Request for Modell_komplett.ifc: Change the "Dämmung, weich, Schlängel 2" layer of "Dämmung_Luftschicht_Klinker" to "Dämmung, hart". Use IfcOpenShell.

First a look at what the model holds.

```python
import ifcopenshell
import ifcopenshell.util.element

model = ifcopenshell.open("Modell_komplett.ifc")
print(model.schema)
for layer_set in model.by_type("IfcMaterialLayerSet"):
    if layer_set.LayerSetName == "Dämmung_Luftschicht_Klinker":
        for layer in layer_set.MaterialLayers:
            print(layer.id(), layer.Material and layer.Material.Name, layer.LayerThickness, sep=" | ")
        print(len(ifcopenshell.util.element.get_elements_by_material(model, layer_set)), "elements and types use it")
print(sorted(m.Name for m in model.by_type("IfcMaterial") if m.Name)[:60])
```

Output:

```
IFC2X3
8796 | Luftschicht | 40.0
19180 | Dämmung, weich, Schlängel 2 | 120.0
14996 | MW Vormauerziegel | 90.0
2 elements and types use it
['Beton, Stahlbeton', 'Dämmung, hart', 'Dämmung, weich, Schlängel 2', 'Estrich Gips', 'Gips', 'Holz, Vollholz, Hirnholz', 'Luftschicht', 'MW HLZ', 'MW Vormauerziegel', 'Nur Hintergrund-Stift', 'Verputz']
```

```python
import ifcopenshell
import ifcopenshell.api.material

model = ifcopenshell.open("Modell_komplett.ifc")

layer_set = next(s for s in model.by_type("IfcMaterialLayerSet") if s.LayerSetName == "Dämmung_Luftschicht_Klinker")
layer = next(l for l in layer_set.MaterialLayers if l.Material and l.Material.Name == "Dämmung, weich, Schlängel 2")
material = next(m for m in model.by_type("IfcMaterial") if m.Name == "Dämmung, hart")

# Point this one layer at the other material; renaming the old one would change it everywhere.
ifcopenshell.api.material.edit_layer(model, layer=layer, attributes={}, material=material)

print([l.Material.Name if l.Material else None for l in layer_set.MaterialLayers])

model.write("Modell_komplett_v2.ifc")
```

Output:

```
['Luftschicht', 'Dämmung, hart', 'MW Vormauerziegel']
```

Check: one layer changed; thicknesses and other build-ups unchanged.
